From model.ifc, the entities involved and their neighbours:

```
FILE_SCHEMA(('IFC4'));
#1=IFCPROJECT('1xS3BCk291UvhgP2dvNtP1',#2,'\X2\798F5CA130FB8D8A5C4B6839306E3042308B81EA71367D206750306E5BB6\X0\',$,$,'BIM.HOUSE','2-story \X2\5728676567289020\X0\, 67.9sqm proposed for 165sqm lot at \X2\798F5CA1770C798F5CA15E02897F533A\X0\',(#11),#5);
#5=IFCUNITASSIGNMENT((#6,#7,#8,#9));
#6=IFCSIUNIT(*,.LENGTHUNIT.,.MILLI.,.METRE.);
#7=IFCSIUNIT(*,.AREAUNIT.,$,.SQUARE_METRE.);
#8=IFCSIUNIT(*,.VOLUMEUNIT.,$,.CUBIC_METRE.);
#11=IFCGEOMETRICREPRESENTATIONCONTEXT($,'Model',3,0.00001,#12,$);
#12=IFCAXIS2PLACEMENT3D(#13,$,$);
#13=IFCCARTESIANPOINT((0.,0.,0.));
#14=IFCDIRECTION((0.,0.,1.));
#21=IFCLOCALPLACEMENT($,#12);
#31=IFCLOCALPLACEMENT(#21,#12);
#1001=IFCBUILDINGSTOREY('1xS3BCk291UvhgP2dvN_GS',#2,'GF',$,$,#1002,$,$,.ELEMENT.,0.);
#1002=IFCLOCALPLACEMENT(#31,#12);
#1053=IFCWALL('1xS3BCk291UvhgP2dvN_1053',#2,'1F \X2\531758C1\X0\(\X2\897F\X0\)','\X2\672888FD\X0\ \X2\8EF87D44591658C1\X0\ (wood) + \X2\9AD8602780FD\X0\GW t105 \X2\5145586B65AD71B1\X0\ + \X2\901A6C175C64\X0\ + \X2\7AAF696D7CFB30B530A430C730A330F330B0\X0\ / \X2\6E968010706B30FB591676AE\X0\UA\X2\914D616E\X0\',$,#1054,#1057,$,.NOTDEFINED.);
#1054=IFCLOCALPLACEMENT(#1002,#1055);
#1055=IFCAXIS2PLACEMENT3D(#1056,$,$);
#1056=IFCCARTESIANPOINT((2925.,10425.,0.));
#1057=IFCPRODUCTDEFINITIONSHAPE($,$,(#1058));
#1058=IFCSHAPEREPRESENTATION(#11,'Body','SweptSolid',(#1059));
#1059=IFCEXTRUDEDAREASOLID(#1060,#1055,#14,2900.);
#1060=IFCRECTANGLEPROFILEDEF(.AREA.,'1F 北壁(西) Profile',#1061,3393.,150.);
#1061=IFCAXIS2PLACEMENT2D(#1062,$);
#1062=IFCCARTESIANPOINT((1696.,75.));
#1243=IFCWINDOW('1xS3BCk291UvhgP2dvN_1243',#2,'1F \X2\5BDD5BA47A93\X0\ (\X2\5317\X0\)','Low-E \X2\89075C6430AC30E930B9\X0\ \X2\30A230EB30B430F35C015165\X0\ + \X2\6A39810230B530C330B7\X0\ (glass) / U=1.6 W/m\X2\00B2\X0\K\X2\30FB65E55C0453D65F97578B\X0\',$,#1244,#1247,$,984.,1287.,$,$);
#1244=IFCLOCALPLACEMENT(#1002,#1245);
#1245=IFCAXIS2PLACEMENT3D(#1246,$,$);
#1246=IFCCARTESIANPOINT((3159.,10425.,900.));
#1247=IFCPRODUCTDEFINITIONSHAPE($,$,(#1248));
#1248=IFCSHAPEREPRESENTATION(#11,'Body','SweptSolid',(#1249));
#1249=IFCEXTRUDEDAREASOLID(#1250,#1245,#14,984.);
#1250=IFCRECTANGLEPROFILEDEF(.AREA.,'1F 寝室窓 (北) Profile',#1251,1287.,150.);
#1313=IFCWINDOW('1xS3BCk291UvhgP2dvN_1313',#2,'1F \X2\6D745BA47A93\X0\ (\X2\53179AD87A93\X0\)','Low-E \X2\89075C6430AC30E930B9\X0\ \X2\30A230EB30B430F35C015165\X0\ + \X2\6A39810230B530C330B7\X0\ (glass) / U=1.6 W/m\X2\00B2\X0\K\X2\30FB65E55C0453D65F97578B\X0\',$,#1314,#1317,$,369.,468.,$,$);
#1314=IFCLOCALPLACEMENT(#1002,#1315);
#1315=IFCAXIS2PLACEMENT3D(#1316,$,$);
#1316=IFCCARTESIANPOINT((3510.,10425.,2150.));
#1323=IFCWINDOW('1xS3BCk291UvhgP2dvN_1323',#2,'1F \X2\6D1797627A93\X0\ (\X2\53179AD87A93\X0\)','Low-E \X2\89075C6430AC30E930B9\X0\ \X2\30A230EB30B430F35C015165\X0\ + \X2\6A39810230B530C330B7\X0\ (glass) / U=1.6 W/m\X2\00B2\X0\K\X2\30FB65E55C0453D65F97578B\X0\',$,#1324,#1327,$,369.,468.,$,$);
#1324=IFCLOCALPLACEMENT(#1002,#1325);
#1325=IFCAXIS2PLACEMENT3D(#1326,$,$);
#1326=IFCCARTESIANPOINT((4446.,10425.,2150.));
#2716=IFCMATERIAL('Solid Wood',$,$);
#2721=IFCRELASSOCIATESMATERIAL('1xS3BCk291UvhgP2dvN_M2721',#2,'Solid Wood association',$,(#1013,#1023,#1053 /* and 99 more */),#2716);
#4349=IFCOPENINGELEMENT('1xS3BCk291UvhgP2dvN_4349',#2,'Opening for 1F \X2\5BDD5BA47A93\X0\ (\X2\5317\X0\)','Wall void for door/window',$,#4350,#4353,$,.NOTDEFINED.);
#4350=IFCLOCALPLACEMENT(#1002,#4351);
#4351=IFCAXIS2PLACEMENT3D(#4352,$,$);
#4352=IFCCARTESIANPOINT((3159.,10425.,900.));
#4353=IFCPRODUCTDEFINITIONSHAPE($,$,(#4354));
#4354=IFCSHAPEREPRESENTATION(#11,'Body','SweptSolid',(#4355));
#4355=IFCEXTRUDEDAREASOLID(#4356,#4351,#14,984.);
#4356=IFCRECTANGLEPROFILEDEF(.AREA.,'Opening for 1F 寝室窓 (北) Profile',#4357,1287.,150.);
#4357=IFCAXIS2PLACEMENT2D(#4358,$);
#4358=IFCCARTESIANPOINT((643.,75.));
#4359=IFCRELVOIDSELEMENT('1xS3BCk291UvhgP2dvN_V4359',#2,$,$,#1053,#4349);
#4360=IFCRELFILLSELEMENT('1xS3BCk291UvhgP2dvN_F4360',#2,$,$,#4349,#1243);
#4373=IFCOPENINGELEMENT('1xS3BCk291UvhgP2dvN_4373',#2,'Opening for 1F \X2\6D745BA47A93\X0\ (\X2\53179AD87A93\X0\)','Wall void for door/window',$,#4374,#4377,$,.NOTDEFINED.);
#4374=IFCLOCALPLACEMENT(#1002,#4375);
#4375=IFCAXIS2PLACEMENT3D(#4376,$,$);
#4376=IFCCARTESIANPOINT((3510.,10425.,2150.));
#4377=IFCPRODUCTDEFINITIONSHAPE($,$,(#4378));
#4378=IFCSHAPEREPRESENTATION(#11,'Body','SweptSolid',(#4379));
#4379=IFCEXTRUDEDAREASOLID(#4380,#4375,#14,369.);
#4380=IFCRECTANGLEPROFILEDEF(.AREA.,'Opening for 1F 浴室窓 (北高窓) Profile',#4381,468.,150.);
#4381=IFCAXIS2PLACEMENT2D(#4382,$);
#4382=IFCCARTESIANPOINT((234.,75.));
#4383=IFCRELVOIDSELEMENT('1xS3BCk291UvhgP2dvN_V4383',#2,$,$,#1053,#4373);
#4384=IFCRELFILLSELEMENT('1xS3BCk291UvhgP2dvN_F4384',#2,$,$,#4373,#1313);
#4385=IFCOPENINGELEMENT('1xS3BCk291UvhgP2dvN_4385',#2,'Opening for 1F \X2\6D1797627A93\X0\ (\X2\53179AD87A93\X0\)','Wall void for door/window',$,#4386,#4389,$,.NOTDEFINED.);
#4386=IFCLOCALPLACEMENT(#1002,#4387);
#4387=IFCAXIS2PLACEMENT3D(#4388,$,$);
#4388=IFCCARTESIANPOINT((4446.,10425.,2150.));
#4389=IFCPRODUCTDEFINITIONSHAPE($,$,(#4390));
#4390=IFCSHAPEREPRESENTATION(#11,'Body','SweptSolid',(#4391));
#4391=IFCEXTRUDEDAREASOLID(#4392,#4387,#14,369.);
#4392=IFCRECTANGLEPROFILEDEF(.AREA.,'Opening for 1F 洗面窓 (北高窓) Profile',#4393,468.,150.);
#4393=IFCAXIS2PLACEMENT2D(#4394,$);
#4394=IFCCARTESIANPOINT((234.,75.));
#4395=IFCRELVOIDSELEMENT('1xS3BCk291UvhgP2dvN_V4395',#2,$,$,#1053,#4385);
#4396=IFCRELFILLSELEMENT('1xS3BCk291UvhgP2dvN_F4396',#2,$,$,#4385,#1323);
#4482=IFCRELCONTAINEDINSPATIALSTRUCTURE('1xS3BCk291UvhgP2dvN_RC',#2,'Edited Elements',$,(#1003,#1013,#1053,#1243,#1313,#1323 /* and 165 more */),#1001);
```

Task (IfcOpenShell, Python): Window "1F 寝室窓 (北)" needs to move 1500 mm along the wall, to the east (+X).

```python
import ifcopenshell
import ifcopenshell.api.geometry
import ifcopenshell.util.placement

model = ifcopenshell.open("model.ifc")

window = model.by_guid("1xS3BCk291UvhgP2dvN_1243")
opening = window.FillsVoids[0].RelatingOpeningElement
wall = opening.VoidsElements[0].RelatingBuildingElement

wall_matrix = ifcopenshell.util.placement.get_local_placement(wall.ObjectPlacement)
shift = wall_matrix[:3, 0] * 1500.0
before = ifcopenshell.util.placement.get_local_placement(window.ObjectPlacement)[:3, 3].copy()

# The window is not placed relative to its opening, so move both.
for product in (opening, window):
    matrix = ifcopenshell.util.placement.get_local_placement(product.ObjectPlacement)
    matrix[:3, 3] += shift
    ifcopenshell.api.geometry.edit_object_placement(model, product=product, matrix=matrix, is_si=False)

after = ifcopenshell.util.placement.get_local_placement(window.ObjectPlacement)[:3, 3]
print("window moved by", (after - before).round(3) + 0.0)

model.write("model_updated.ifc")
```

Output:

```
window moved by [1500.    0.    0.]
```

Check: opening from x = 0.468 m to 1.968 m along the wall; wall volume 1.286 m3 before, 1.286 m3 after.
